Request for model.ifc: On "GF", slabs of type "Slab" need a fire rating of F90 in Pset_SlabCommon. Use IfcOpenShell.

First a look at what the model holds.

```python
import ifcopenshell
import ifcopenshell.util.element

model = ifcopenshell.open("model.ifc")
print(model.schema)
storey = next(s for s in model.by_type("IfcBuildingStorey") if s.Name == "GF")
slabs = [e for e in ifcopenshell.util.element.get_decomposition(storey) if e.is_a("IfcSlab")]
seen = {}
for e in slabs:
    element_type = ifcopenshell.util.element.get_type(e)
    key = (element_type.Name if element_type != e and element_type else None, ifcopenshell.util.element.get_pset(e, "Pset_SlabCommon", "FireRating"))
    seen[key] = seen.get(key, 0) + 1
for (name, value), count in sorted(seen.items(), key=str):
    print(count, "x", name, "|", value)
```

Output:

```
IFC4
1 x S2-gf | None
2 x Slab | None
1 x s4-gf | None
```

```python
import ifcopenshell
import ifcopenshell.api.pset
import ifcopenshell.util.element

model = ifcopenshell.open("model.ifc")

storey = next(s for s in model.by_type("IfcBuildingStorey") if s.Name == "GF")
slabs = [e for e in ifcopenshell.util.element.get_decomposition(storey) if e.is_a("IfcSlab")]

count = 0
for e in slabs:
    element_type = ifcopenshell.util.element.get_type(e)
    if element_type in (None, e) or element_type.Name != "Slab":
        continue
    # add_pset returns the element's existing set when there is one.
    pset = ifcopenshell.api.pset.add_pset(model, product=e, name="Pset_SlabCommon")
    ifcopenshell.api.pset.edit_pset(model, pset=pset, properties={"FireRating": "F90"})
    count += 1

print(count, "slabs updated")

model.write("model_edited.ifc")
```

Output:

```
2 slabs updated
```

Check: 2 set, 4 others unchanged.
